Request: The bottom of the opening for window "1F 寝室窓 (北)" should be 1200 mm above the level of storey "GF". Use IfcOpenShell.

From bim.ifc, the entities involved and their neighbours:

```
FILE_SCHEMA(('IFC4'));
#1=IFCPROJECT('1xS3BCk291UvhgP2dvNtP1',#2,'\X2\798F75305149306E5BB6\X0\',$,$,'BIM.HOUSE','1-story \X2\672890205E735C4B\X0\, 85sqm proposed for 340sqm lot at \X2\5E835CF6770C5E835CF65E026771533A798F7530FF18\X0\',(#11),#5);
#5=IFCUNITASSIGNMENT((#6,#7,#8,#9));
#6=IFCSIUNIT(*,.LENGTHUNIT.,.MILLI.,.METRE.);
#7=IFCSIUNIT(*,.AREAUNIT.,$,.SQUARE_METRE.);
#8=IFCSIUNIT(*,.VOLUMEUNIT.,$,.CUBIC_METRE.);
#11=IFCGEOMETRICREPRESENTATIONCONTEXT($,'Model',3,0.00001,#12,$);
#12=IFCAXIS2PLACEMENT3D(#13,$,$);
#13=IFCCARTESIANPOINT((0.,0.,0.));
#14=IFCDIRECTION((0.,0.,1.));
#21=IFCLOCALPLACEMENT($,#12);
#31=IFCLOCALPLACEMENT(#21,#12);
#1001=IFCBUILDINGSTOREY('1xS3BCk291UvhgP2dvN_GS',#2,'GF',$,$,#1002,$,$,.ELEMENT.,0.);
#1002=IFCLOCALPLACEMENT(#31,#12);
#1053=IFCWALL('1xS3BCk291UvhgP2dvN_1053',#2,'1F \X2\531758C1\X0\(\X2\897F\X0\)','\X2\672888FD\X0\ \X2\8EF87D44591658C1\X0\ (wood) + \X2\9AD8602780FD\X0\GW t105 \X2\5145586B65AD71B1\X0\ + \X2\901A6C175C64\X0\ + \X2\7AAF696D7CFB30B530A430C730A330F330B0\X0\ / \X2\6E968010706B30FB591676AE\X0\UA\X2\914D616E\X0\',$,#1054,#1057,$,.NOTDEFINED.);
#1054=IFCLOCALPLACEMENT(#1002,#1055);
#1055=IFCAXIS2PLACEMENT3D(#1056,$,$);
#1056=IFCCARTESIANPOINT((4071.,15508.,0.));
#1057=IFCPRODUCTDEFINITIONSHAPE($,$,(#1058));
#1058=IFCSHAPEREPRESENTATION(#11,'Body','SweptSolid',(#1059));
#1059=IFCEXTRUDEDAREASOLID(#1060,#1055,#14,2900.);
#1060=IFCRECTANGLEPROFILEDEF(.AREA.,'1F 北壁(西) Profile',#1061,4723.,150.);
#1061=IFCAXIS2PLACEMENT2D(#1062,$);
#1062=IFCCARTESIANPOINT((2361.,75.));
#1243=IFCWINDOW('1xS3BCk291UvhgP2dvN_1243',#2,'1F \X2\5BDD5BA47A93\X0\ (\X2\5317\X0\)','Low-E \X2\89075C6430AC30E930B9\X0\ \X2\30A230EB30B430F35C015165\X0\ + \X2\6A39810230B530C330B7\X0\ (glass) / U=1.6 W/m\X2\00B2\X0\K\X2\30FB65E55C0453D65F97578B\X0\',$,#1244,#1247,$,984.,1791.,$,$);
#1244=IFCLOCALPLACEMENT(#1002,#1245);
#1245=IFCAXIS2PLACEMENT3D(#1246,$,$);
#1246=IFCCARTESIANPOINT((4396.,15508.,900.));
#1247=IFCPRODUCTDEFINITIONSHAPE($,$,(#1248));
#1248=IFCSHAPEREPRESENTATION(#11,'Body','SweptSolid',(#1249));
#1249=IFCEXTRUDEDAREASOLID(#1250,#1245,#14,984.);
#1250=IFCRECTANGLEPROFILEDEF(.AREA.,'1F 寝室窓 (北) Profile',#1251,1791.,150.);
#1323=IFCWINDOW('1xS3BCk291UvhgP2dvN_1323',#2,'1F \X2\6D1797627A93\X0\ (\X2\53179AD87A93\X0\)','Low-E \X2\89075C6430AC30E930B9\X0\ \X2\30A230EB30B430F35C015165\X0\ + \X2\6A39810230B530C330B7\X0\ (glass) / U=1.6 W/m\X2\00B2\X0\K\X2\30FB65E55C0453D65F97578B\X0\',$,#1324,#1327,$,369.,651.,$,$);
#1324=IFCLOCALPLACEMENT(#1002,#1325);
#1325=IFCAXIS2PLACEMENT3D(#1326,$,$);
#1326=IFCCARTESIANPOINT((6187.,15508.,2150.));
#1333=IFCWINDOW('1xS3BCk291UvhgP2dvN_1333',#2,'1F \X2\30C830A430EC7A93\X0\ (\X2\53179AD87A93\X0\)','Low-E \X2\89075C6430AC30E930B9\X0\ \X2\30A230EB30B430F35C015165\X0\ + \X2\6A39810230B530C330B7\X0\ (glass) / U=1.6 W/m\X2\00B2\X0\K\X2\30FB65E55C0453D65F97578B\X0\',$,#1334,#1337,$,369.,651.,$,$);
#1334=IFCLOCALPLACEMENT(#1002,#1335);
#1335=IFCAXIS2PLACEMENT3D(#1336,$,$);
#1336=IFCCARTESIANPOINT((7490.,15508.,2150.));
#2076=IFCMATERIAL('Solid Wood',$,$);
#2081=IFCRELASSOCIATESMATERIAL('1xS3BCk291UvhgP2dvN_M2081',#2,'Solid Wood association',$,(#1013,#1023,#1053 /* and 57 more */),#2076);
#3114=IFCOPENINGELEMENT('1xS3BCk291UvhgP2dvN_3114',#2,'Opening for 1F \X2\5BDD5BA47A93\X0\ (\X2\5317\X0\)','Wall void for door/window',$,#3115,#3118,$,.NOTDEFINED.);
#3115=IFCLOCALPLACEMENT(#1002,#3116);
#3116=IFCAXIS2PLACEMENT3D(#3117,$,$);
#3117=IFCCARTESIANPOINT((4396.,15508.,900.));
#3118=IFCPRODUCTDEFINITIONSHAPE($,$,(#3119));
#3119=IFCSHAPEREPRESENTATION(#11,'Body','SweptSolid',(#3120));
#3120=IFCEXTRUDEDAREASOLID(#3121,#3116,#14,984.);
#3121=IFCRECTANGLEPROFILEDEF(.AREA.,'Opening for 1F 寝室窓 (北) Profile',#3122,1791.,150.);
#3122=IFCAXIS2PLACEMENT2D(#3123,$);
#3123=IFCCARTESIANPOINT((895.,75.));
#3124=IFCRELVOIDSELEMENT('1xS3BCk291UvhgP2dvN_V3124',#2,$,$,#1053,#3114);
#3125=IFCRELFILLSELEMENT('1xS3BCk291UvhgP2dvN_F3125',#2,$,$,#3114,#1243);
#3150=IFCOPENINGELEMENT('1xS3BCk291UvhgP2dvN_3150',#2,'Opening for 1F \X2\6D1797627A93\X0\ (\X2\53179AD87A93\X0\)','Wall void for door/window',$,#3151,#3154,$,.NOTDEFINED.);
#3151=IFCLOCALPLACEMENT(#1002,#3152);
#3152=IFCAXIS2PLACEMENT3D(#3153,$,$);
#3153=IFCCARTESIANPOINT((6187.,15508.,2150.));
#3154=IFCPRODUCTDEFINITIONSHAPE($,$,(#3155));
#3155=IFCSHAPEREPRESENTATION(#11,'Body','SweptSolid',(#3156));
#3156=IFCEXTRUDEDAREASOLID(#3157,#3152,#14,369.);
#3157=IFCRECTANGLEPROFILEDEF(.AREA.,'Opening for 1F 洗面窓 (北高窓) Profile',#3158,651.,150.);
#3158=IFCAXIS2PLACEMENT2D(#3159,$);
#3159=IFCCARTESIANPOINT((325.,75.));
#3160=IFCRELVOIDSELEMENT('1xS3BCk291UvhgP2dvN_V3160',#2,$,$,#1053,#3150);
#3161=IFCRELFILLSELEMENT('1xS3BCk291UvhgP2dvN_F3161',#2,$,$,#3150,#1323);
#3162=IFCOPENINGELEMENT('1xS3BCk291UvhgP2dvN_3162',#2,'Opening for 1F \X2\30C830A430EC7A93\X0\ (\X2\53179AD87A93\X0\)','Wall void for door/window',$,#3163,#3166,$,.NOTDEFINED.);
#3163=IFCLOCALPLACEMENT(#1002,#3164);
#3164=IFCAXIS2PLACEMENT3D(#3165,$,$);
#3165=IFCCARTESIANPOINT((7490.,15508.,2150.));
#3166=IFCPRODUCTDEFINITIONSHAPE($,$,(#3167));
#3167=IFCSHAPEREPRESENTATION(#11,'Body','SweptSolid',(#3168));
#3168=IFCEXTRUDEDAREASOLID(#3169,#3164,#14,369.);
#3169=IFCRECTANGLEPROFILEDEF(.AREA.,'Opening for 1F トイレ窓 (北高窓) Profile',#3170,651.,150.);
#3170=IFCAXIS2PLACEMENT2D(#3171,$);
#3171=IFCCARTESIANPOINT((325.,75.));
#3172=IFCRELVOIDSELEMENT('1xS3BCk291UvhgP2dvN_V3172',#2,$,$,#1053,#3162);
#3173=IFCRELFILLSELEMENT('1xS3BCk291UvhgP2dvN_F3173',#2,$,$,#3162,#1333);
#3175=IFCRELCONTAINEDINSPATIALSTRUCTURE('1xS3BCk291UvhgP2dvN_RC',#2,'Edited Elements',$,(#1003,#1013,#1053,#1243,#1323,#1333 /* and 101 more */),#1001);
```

```python
import numpy as np
import ifcopenshell
import ifcopenshell.api.geometry
import ifcopenshell.geom
import ifcopenshell.util.element
import ifcopenshell.util.placement
import ifcopenshell.util.shape
import ifcopenshell.util.unit

model = ifcopenshell.open("bim.ifc")
unit_scale = ifcopenshell.util.unit.calculate_unit_scale(model)

window = model.by_guid("1xS3BCk291UvhgP2dvN_1243")
opening = window.FillsVoids[0].RelatingOpeningElement
storey = ifcopenshell.util.element.get_container(window, ifc_class="IfcBuildingStorey")
level = ifcopenshell.util.placement.get_local_placement(storey.ObjectPlacement)[2, 3]

# The opening's origin need not be at the sill, so measure its lowest point.
shape = ifcopenshell.geom.create_shape(ifcopenshell.geom.settings(), opening)
bottom = ifcopenshell.util.shape.get_shape_bottom_elevation(shape, shape.geometry) / unit_scale
dz = level + 1200.0 - bottom

shift = np.array([0.0, 0.0, dz])
# The window is not placed relative to its opening, so move both.
for product in (opening, window):
    matrix = ifcopenshell.util.placement.get_local_placement(product.ObjectPlacement)
    matrix[:3, 3] += shift
    ifcopenshell.api.geometry.edit_object_placement(model, product=product, matrix=matrix, is_si=False)

print(f"moved by {dz * unit_scale:+.3f} m")

model.write("bim_updated.ifc")
```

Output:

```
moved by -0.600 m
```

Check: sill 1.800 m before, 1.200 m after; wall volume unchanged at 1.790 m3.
